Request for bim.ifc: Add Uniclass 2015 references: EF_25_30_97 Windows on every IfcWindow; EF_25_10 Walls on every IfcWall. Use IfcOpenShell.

First a look at what the model holds.

```python
import ifcopenshell

model = ifcopenshell.open("bim.ifc")
print(model.schema)
print("classifications:", [c.Name for c in model.by_type("IfcClassification")])
for ifc_class in ("IfcDoor", "IfcRoof", "IfcStair", "IfcWall", "IfcWindow"):
    print(ifc_class, len(model.by_type(ifc_class)))
```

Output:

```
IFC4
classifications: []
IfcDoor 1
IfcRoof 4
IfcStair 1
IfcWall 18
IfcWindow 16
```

```python
import ifcopenshell
import ifcopenshell.api.classification

model = ifcopenshell.open("bim.ifc")

system = ifcopenshell.api.classification.add_classification(model, classification="Uniclass 2015")

codes = {
    "IfcWindow": ("EF_25_30_97", "Windows"),
    "IfcWall": ("EF_25_10", "Walls"),
}
for ifc_class, (code, name) in codes.items():
    products = model.by_type(ifc_class)
    ifcopenshell.api.classification.add_reference(
        model, products=products, classification=system, identification=code, name=name
    )
    print(code, len(products))

model.write("bim_updated.ifc")
```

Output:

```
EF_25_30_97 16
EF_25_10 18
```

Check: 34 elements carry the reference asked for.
